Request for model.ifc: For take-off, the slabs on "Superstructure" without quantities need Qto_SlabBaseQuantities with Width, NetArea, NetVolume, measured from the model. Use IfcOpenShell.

First a look at what the model holds.

```python
import ifcopenshell
import ifcopenshell.util.element
import ifcopenshell.util.unit

model = ifcopenshell.open("model.ifc")
print(model.schema)
for unit_type in ("LENGTHUNIT", "AREAUNIT", "VOLUMEUNIT"):
    print(unit_type, ifcopenshell.util.unit.calculate_unit_scale(model, unit_type))
storey = next(s for s in model.by_type("IfcBuildingStorey") if s.Name == "Superstructure")
slabs = [e for e in ifcopenshell.util.element.get_decomposition(storey) if e.is_a("IfcSlab")]
for e in sorted(slabs, key=lambda e: e.id()):
    print(e.id(), e.is_a(), e.Name, list(ifcopenshell.util.element.get_psets(e, qtos_only=True)), sep=" | ")
```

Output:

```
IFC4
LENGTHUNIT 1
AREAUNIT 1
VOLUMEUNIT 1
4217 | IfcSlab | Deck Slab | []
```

```python
import ifcopenshell
import ifcopenshell.api.pset
import ifcopenshell.geom
import ifcopenshell.util.element
import ifcopenshell.util.shape
import ifcopenshell.util.unit

model = ifcopenshell.open("model.ifc")
unit_scale = ifcopenshell.util.unit.calculate_unit_scale(model)
area_scale = ifcopenshell.util.unit.calculate_unit_scale(model, "AREAUNIT")
volume_scale = ifcopenshell.util.unit.calculate_unit_scale(model, "VOLUMEUNIT")
settings = ifcopenshell.geom.settings()

storey = next(s for s in model.by_type("IfcBuildingStorey") if s.Name == "Superstructure")
slabs = [e for e in ifcopenshell.util.element.get_decomposition(storey) if e.is_a("IfcSlab")]

for e in sorted(slabs, key=lambda e: e.id()):
    if ifcopenshell.util.element.get_psets(e, qtos_only=True, should_inherit=False):
        continue
    # Geometry comes back in metres, in the element's own axes.
    shape = ifcopenshell.geom.create_shape(settings, e)
    values = {
        "Width": ifcopenshell.util.shape.get_z(shape.geometry) / unit_scale,
        "NetArea": ifcopenshell.util.shape.get_footprint_area(shape.geometry) / area_scale,
        "NetVolume": ifcopenshell.util.shape.get_volume(shape.geometry) / volume_scale,
    }
    qto = ifcopenshell.api.pset.add_qto(model, product=e, name="Qto_SlabBaseQuantities")
    ifcopenshell.api.pset.edit_qto(model, qto=qto, properties=values)
    print(e.id(), {k: round(v, 3) for k, v in values.items()})

model.write("model_updated.ifc")
```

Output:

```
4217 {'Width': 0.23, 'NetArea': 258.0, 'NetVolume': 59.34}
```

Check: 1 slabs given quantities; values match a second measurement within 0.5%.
